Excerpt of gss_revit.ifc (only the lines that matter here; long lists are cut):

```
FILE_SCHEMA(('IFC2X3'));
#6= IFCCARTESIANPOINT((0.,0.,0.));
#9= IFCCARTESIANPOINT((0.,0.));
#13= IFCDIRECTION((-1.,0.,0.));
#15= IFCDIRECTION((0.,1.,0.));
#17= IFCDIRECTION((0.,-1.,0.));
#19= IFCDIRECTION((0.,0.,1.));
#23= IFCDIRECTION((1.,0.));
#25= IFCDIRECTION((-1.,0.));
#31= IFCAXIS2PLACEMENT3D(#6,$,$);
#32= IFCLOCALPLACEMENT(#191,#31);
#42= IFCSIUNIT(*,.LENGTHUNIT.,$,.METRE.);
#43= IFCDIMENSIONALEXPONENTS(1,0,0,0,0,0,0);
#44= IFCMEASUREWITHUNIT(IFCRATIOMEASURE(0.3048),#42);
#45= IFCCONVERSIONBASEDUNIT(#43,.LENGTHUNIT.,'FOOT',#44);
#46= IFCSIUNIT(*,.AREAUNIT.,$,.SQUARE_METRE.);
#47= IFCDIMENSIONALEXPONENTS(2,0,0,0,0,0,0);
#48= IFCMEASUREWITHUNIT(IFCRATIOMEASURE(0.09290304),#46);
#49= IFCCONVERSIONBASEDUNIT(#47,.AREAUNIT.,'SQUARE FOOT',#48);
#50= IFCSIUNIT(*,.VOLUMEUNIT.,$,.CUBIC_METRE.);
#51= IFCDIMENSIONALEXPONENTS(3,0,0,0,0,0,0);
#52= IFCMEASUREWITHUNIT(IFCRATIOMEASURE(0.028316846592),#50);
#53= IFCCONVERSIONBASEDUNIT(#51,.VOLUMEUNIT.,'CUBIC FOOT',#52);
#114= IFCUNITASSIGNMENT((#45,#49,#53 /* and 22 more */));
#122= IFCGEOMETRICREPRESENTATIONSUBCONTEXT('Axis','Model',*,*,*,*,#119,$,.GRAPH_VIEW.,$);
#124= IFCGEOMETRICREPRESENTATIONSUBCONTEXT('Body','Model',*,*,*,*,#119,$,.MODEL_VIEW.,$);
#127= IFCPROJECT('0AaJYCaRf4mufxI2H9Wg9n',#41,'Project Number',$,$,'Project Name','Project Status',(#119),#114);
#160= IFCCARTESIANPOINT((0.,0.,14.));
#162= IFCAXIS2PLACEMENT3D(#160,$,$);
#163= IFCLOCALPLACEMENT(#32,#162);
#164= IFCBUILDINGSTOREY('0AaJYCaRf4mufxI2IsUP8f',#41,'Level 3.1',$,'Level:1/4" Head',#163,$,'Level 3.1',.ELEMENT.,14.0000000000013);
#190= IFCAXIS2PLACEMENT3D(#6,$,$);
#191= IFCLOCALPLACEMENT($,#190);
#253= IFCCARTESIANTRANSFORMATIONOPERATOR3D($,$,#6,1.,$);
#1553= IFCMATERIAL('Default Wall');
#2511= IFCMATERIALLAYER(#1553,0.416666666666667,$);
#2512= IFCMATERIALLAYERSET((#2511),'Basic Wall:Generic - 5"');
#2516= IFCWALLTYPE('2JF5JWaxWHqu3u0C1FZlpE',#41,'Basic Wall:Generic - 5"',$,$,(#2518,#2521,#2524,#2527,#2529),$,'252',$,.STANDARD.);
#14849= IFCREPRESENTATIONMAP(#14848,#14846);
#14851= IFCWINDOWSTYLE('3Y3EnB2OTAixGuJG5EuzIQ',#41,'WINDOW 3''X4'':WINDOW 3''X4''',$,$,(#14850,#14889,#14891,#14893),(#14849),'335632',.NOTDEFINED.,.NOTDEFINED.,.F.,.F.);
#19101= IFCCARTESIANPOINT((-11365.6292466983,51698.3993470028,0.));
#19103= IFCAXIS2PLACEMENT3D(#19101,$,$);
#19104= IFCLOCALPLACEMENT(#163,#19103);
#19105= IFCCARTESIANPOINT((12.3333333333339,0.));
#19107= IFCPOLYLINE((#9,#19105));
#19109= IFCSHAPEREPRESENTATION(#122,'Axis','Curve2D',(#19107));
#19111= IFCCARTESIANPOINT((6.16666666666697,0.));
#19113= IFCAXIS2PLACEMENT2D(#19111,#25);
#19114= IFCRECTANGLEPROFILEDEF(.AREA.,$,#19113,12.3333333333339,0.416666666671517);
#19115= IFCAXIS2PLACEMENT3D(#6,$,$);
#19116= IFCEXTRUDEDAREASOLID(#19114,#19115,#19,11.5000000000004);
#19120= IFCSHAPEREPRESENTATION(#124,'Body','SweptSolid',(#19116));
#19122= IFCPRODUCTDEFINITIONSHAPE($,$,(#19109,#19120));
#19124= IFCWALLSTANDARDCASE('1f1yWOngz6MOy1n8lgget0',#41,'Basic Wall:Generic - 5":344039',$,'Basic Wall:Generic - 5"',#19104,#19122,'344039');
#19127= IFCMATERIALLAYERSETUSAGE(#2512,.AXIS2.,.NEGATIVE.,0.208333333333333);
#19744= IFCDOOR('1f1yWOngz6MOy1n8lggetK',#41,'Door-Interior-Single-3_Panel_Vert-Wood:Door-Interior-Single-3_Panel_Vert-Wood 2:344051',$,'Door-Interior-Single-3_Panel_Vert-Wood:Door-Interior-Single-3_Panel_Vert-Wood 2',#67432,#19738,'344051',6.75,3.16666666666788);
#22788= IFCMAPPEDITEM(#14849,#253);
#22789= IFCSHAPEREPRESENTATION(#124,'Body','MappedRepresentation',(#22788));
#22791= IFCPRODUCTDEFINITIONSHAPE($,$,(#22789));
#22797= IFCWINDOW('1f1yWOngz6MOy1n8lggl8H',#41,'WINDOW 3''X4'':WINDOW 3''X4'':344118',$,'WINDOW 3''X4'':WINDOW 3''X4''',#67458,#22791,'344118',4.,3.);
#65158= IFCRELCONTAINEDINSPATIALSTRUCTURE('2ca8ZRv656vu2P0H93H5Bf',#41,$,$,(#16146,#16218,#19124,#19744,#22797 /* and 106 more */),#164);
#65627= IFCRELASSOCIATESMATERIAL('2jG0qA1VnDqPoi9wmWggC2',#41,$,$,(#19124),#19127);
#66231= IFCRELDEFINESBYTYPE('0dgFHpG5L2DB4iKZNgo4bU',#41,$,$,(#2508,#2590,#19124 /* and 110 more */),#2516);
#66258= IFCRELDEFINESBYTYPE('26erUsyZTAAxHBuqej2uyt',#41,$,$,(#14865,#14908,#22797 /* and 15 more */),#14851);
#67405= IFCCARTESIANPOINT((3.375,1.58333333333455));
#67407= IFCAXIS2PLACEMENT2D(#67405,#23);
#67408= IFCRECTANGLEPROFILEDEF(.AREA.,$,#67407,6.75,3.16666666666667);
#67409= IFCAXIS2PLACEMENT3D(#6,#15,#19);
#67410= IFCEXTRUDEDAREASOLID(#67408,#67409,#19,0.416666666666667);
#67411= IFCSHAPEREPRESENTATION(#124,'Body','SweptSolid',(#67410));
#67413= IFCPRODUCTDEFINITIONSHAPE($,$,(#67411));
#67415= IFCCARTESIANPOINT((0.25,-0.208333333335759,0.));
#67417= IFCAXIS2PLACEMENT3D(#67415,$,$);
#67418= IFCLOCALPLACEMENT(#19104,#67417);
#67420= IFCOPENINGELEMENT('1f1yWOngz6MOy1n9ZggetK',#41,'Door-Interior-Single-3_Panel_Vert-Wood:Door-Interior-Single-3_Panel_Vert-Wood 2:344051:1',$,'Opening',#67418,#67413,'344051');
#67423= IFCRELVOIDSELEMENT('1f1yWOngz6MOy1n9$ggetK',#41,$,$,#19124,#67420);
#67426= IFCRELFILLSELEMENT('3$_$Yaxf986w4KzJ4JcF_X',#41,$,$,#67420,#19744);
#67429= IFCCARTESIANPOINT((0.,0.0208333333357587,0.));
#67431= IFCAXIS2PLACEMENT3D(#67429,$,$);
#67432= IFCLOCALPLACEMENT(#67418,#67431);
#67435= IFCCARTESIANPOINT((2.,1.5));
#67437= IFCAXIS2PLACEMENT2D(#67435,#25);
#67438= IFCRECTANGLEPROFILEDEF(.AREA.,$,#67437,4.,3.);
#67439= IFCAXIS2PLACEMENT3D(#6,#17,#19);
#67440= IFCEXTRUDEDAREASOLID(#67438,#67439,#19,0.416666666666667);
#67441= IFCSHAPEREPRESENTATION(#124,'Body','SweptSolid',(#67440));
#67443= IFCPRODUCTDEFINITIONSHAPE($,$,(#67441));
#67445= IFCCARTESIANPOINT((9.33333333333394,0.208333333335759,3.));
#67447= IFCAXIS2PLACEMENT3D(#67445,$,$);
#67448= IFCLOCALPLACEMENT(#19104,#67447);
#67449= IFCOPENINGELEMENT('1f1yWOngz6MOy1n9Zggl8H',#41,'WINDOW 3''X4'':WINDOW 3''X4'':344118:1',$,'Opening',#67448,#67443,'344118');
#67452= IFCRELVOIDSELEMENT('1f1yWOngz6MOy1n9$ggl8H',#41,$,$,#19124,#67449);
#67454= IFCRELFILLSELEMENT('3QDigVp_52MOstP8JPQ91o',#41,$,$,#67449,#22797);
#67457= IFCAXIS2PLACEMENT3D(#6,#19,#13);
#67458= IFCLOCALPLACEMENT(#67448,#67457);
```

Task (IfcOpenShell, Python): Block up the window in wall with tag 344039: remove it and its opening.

```python
import ifcopenshell
import ifcopenshell.api.feature
import ifcopenshell.api.root
import ifcopenshell.geom
import ifcopenshell.util.shape

model = ifcopenshell.open("gss_revit.ifc")
settings = ifcopenshell.geom.settings()


def volume(element):
    """Net volume in cubic metres, openings subtracted."""
    shape = ifcopenshell.geom.create_shape(settings, element)
    return ifcopenshell.util.shape.get_volume(shape.geometry)


window = model.by_id(22797)
opening = window.FillsVoids[0].RelatingOpeningElement
wall = opening.VoidsElements[0].RelatingBuildingElement
before = volume(wall)

ifcopenshell.api.root.remove_product(model, product=window)
ifcopenshell.api.feature.remove_feature(model, feature=opening)

after = volume(wall)

print(f"wall volume {before:.3f} -> {after:.3f} m3")

model.write("gss_revit_updated.ifc")
```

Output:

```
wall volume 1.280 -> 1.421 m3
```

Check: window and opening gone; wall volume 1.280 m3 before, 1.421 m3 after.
